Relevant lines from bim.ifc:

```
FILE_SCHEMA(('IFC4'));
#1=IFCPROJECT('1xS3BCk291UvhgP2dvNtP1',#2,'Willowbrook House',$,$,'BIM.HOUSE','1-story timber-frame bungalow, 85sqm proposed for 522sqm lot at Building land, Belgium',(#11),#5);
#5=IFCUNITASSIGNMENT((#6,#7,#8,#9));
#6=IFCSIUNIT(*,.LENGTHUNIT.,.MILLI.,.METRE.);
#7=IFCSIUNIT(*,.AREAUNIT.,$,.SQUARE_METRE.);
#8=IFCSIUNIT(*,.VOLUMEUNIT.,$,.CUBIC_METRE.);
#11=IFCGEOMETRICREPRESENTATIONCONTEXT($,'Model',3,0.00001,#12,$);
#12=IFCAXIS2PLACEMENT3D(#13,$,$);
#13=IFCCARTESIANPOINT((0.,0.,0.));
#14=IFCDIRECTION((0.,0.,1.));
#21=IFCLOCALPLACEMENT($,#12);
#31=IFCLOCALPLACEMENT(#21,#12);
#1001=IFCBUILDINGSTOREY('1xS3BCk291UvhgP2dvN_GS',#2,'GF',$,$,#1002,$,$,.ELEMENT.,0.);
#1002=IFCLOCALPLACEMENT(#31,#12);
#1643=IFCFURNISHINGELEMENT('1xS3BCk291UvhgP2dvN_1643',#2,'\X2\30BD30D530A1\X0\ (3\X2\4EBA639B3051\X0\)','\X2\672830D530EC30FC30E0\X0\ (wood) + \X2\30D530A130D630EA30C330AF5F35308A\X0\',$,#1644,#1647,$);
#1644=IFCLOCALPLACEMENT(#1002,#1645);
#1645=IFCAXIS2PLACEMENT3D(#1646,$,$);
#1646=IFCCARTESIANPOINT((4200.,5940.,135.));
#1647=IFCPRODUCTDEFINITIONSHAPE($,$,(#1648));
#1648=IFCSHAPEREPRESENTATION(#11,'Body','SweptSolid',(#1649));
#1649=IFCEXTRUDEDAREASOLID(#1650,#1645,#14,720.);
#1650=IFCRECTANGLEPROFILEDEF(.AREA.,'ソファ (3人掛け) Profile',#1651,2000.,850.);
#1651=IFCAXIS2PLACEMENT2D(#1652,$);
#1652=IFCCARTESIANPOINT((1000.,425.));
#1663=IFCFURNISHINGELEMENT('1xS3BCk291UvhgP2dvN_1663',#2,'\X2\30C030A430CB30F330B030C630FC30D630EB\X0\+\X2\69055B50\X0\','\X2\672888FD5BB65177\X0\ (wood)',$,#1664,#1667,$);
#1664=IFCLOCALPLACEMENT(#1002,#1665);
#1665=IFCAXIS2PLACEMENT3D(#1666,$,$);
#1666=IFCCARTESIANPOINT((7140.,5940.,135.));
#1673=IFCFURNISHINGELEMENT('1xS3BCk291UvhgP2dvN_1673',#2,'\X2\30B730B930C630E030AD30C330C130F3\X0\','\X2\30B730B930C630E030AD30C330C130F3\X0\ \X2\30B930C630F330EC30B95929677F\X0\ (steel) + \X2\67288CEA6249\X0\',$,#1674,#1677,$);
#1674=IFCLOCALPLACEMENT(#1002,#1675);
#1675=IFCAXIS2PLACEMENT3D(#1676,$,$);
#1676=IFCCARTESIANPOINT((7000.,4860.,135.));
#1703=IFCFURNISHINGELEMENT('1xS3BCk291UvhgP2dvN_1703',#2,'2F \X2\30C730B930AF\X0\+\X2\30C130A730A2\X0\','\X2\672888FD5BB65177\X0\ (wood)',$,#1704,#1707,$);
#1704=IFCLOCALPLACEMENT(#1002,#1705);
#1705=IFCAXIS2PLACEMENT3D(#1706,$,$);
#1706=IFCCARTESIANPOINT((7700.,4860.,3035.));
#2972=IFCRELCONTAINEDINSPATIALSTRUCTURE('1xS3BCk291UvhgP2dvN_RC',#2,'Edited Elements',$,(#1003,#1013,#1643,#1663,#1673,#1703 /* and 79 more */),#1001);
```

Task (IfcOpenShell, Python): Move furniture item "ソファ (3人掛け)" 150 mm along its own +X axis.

```python
import ifcopenshell
import ifcopenshell.api.geometry
import ifcopenshell.util.placement

model = ifcopenshell.open("bim.ifc")

item = model.by_guid("1xS3BCk291UvhgP2dvN_1643")
matrix = ifcopenshell.util.placement.get_local_placement(item.ObjectPlacement)
matrix[:3, 3] += matrix[:3, 0] * 150.0
ifcopenshell.api.geometry.edit_object_placement(model, product=item, matrix=matrix, is_si=False)

print(ifcopenshell.util.placement.get_local_placement(item.ObjectPlacement).round(3) + 0.0)

model.write("bim_rev.ifc")
```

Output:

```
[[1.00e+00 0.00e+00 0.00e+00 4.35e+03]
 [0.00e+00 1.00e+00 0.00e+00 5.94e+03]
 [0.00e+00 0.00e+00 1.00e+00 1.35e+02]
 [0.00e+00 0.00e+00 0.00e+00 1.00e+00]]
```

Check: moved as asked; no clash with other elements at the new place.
